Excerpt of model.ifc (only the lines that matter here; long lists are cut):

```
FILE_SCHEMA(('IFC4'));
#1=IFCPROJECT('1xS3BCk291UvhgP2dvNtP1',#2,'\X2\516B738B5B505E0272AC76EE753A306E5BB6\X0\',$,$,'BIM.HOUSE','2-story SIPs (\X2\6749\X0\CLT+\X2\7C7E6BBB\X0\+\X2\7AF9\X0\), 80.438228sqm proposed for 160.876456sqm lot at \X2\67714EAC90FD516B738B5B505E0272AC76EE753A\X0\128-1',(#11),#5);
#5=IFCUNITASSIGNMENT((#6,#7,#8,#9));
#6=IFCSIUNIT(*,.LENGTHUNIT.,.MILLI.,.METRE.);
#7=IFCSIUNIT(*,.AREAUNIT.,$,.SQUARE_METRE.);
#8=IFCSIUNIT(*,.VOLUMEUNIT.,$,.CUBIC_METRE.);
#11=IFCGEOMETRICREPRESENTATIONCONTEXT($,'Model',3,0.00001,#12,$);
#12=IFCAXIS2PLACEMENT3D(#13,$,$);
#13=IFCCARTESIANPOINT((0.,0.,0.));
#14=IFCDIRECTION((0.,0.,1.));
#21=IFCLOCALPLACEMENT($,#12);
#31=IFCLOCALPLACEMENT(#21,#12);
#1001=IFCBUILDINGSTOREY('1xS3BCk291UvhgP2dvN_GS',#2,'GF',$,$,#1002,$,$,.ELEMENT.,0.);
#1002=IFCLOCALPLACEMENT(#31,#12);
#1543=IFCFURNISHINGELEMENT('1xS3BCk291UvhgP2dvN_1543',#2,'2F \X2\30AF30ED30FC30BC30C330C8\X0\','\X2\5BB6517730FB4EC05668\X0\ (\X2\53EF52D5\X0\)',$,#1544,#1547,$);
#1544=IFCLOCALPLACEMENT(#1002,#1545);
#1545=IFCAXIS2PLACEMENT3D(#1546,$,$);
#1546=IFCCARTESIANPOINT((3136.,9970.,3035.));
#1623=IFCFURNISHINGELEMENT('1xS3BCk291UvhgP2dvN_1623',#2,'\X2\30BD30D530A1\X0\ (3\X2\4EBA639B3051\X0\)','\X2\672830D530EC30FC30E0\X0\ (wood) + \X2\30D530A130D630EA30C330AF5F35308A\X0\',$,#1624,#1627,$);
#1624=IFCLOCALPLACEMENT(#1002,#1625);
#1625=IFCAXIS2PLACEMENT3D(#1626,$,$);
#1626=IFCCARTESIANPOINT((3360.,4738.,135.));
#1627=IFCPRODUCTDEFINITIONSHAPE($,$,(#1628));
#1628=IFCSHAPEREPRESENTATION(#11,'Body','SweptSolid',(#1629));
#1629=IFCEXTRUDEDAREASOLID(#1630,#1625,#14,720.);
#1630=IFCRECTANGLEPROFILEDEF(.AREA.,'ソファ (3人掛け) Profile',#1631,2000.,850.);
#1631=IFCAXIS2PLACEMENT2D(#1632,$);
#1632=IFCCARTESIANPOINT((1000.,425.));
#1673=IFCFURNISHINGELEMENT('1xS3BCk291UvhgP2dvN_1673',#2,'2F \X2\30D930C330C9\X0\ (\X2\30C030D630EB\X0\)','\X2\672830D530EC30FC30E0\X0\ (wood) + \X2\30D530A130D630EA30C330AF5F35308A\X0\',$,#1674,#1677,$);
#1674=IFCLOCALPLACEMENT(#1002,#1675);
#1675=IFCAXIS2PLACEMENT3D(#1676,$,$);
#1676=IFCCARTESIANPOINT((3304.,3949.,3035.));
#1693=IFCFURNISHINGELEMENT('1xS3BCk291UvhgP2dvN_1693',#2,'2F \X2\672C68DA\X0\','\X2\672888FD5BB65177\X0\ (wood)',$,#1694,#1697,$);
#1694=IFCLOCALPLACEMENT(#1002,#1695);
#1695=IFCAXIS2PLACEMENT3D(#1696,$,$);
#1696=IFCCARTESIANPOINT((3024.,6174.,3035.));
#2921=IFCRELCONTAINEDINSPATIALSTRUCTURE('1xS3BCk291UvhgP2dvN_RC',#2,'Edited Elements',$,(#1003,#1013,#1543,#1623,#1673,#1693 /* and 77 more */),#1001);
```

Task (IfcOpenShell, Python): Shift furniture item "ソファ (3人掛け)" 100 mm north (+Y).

```python
import ifcopenshell
import ifcopenshell.api.geometry
import ifcopenshell.util.placement
import ifcopenshell.util.unit

model = ifcopenshell.open("model.ifc")
unit_scale = ifcopenshell.util.unit.calculate_unit_scale(model)

item = model.by_guid("1xS3BCk291UvhgP2dvN_1623")
matrix = ifcopenshell.util.placement.get_local_placement(item.ObjectPlacement)
matrix[1, 3] += 0.1 / unit_scale
ifcopenshell.api.geometry.edit_object_placement(model, product=item, matrix=matrix, is_si=False)

print(ifcopenshell.util.placement.get_local_placement(item.ObjectPlacement).round(3) + 0.0)

model.write("model_v2.ifc")
```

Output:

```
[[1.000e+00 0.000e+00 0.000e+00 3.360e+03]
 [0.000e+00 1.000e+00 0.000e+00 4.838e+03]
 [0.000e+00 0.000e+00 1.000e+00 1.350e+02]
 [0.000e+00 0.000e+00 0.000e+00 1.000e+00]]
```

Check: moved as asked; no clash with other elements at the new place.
